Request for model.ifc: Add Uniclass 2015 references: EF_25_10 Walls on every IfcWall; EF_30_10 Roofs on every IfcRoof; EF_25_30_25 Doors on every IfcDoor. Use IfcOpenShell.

First a look at what the model holds.

```python
import ifcopenshell

model = ifcopenshell.open("model.ifc")
print(model.schema)
print("classifications:", [c.Name for c in model.by_type("IfcClassification")])
for ifc_class in ("IfcDoor", "IfcRoof", "IfcStair", "IfcWall", "IfcWindow"):
    print(ifc_class, len(model.by_type(ifc_class)))
```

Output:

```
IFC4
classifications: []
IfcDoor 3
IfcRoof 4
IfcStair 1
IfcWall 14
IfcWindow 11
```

```python
import ifcopenshell
import ifcopenshell.api.classification

model = ifcopenshell.open("model.ifc")

system = ifcopenshell.api.classification.add_classification(model, classification="Uniclass 2015")

codes = {
    "IfcWall": ("EF_25_10", "Walls"),
    "IfcRoof": ("EF_30_10", "Roofs"),
    "IfcDoor": ("EF_25_30_25", "Doors"),
}
for ifc_class, (code, name) in codes.items():
    products = model.by_type(ifc_class)
    ifcopenshell.api.classification.add_reference(
        model, products=products, classification=system, identification=code, name=name
    )
    print(code, len(products))

model.write("model_rev.ifc")
```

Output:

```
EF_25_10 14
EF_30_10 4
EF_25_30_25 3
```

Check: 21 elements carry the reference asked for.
